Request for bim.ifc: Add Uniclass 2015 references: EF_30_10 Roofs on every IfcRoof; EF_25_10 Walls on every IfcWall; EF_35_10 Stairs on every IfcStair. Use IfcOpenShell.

First a look at what the model holds.

```python
import ifcopenshell

model = ifcopenshell.open("bim.ifc")
print(model.schema)
print("classifications:", [c.Name for c in model.by_type("IfcClassification")])
for ifc_class in ("IfcDoor", "IfcRoof", "IfcStair", "IfcWall", "IfcWindow"):
    print(ifc_class, len(model.by_type(ifc_class)))
```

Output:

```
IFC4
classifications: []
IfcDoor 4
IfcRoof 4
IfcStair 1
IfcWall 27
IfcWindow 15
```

```python
import ifcopenshell
import ifcopenshell.api.classification

model = ifcopenshell.open("bim.ifc")

system = ifcopenshell.api.classification.add_classification(model, classification="Uniclass 2015")

codes = {
    "IfcRoof": ("EF_30_10", "Roofs"),
    "IfcWall": ("EF_25_10", "Walls"),
    "IfcStair": ("EF_35_10", "Stairs"),
}
for ifc_class, (code, name) in codes.items():
    products = model.by_type(ifc_class)
    ifcopenshell.api.classification.add_reference(
        model, products=products, classification=system, identification=code, name=name
    )
    print(code, len(products))

model.write("bim_rev.ifc")
```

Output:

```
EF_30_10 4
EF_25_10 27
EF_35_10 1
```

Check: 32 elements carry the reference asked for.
